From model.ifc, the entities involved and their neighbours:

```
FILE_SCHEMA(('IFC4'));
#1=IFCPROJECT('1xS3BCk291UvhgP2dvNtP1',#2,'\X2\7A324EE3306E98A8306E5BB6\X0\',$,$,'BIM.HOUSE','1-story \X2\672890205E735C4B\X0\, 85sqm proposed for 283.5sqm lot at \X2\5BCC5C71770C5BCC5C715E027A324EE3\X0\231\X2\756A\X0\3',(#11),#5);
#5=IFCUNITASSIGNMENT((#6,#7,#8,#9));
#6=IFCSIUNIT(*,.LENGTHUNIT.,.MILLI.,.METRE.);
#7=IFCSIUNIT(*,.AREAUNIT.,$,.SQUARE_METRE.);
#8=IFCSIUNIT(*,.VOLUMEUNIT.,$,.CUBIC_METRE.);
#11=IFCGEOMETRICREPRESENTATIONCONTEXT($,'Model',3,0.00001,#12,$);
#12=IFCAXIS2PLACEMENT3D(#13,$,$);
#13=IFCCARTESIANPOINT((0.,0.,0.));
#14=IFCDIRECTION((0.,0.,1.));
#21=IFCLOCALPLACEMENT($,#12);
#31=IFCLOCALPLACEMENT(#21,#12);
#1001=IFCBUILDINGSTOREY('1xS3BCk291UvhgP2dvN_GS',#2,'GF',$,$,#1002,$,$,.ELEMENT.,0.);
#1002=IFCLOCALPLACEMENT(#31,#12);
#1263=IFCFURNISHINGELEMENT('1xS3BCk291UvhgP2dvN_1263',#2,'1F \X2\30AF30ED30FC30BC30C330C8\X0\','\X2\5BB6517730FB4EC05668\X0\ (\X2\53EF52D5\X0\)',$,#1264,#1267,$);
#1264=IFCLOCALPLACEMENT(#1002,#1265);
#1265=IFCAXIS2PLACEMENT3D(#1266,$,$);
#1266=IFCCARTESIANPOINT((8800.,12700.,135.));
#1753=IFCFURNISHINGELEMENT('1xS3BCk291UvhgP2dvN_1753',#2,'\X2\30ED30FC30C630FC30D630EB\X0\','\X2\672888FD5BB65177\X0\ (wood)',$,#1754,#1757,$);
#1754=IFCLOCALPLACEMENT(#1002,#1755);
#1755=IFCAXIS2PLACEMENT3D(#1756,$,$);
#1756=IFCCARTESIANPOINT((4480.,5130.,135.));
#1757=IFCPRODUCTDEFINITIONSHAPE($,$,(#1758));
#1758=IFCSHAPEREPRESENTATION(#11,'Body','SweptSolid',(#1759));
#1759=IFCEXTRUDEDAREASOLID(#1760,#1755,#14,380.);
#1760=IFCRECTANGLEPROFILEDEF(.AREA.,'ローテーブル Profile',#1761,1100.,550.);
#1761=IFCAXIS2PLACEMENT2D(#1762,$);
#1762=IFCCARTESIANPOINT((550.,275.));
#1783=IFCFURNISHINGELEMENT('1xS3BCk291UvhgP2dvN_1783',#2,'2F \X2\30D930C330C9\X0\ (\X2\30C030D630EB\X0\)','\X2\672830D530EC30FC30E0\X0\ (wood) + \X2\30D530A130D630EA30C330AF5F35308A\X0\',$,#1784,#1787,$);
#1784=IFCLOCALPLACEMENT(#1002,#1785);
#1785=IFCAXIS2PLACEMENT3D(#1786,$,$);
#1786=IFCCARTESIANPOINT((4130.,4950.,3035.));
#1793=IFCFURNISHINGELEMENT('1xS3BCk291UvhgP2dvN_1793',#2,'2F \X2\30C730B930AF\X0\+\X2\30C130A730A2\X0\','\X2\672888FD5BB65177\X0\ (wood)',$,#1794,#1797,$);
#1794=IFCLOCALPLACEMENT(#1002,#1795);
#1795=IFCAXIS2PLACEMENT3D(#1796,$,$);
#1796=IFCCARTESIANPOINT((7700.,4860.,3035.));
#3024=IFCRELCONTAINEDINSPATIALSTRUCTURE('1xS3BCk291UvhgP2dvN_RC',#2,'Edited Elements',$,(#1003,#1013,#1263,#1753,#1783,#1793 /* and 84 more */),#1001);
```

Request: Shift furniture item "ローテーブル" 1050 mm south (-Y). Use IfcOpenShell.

```python
import ifcopenshell
import ifcopenshell.api.geometry
import ifcopenshell.util.placement
import ifcopenshell.util.unit

model = ifcopenshell.open("model.ifc")
unit_scale = ifcopenshell.util.unit.calculate_unit_scale(model)

item = model.by_guid("1xS3BCk291UvhgP2dvN_1753")
matrix = ifcopenshell.util.placement.get_local_placement(item.ObjectPlacement)
matrix[1, 3] -= 1.05 / unit_scale
ifcopenshell.api.geometry.edit_object_placement(model, product=item, matrix=matrix, is_si=False)

print(ifcopenshell.util.placement.get_local_placement(item.ObjectPlacement).round(3) + 0.0)

model.write("model_v2.ifc")
```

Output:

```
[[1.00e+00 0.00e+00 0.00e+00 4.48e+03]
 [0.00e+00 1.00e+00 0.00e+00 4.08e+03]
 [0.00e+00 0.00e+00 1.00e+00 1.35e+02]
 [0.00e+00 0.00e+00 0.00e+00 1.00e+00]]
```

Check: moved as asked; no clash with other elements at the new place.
